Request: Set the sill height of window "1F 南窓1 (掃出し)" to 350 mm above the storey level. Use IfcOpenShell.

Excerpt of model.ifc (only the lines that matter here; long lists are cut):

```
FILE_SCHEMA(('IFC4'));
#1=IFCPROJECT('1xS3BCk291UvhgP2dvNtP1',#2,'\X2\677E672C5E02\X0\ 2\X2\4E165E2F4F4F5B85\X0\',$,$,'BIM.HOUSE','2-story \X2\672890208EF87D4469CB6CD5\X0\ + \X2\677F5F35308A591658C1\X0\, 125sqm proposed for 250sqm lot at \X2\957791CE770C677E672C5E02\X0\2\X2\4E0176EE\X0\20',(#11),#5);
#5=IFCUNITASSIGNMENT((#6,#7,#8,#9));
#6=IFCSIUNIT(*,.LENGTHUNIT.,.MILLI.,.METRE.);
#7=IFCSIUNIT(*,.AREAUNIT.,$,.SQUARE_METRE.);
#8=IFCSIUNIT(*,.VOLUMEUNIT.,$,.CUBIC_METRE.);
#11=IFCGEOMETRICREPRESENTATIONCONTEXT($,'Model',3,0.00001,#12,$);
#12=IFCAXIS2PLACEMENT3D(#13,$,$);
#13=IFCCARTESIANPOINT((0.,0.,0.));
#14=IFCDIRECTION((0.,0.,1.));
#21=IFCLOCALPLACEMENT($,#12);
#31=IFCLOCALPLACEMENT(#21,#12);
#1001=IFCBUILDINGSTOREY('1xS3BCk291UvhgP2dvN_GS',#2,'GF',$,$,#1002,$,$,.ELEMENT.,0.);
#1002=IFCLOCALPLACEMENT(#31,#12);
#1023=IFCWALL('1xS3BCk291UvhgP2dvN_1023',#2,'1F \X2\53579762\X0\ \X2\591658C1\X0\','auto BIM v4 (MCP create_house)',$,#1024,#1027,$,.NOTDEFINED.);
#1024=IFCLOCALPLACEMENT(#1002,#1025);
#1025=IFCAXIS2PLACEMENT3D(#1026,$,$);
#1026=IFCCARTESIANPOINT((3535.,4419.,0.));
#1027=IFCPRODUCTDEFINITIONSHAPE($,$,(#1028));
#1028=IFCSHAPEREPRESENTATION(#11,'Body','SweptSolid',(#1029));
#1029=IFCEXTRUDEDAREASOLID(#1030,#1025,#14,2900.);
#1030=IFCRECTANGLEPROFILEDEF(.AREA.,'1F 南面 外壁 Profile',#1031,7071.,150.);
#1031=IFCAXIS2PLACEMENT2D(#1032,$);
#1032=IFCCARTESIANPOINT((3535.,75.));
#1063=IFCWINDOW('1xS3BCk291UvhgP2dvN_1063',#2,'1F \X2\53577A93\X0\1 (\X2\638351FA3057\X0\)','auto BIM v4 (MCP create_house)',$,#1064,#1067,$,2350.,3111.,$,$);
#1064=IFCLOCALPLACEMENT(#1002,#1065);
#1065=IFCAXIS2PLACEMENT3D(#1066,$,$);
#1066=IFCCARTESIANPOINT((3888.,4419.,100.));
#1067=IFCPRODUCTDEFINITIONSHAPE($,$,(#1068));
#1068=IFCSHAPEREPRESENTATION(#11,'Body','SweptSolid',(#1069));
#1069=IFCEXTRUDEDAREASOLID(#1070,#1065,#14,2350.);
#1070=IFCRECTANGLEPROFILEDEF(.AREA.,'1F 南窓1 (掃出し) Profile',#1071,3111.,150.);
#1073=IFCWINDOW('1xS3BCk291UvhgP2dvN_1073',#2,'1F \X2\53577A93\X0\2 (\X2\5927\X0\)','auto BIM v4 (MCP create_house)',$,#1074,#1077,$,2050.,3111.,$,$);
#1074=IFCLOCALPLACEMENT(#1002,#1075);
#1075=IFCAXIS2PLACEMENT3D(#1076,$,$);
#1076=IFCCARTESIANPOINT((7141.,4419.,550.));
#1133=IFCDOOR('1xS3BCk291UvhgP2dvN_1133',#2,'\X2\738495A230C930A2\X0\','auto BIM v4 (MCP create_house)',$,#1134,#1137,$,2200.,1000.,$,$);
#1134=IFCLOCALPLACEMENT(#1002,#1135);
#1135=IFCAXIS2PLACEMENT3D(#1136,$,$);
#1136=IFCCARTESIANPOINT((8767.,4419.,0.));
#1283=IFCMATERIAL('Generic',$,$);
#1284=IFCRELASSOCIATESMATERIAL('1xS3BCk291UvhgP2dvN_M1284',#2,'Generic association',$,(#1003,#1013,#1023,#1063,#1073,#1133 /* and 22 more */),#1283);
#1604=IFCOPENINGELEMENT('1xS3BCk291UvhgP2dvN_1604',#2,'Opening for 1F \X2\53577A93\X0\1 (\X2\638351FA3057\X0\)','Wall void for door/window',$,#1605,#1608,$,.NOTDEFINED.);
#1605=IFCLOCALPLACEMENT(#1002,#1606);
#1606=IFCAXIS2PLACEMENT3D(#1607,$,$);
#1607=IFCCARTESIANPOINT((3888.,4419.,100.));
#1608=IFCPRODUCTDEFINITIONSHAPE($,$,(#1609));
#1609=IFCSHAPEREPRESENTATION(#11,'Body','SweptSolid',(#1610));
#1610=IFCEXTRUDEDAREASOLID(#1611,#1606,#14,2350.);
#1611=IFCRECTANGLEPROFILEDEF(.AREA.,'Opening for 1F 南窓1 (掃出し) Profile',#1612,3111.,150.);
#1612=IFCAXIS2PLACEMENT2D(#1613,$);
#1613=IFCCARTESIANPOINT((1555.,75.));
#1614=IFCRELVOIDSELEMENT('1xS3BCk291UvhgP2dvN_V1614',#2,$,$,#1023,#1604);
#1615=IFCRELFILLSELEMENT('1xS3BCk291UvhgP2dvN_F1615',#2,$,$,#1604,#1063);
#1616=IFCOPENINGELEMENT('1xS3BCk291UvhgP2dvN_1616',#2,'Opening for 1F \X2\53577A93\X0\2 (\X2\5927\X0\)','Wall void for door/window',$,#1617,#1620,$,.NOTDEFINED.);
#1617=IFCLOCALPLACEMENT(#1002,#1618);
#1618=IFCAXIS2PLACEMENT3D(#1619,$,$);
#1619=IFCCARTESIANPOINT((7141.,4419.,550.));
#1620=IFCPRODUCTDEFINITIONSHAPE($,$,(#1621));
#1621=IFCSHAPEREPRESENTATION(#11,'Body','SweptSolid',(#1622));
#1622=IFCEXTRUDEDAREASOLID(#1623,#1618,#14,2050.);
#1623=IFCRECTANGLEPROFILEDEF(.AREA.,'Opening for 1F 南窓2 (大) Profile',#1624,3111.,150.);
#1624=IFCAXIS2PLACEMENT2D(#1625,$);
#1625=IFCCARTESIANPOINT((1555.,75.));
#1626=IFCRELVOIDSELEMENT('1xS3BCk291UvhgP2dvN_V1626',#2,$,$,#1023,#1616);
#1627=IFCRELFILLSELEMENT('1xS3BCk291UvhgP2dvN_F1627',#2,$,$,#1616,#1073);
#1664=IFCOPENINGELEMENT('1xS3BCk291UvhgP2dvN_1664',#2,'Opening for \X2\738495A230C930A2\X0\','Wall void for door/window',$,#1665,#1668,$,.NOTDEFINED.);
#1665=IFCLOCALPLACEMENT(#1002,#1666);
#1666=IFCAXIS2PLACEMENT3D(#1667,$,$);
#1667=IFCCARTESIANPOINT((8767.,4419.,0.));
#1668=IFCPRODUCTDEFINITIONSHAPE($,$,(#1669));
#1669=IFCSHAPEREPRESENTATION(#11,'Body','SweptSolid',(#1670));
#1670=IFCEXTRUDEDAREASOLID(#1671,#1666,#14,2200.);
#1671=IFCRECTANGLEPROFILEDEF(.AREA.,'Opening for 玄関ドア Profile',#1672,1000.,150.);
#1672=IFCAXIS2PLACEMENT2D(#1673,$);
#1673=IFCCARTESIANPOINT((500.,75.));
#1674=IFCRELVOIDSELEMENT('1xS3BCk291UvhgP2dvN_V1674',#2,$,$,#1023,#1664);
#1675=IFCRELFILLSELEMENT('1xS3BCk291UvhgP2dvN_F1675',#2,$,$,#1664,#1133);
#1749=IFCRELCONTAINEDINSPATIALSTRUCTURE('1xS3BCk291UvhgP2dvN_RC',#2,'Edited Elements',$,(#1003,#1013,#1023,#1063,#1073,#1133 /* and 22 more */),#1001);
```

```python
import numpy as np
import ifcopenshell
import ifcopenshell.api.geometry
import ifcopenshell.geom
import ifcopenshell.util.element
import ifcopenshell.util.placement
import ifcopenshell.util.shape
import ifcopenshell.util.unit

model = ifcopenshell.open("model.ifc")
unit_scale = ifcopenshell.util.unit.calculate_unit_scale(model)

window = model.by_id(1063)
opening = window.FillsVoids[0].RelatingOpeningElement
storey = ifcopenshell.util.element.get_container(window, ifc_class="IfcBuildingStorey")
level = ifcopenshell.util.placement.get_local_placement(storey.ObjectPlacement)[2, 3]

# The opening's origin need not be at the sill, so measure its lowest point.
shape = ifcopenshell.geom.create_shape(ifcopenshell.geom.settings(), opening)
bottom = ifcopenshell.util.shape.get_shape_bottom_elevation(shape, shape.geometry) / unit_scale
dz = level + 350.0 - bottom

shift = np.array([0.0, 0.0, dz])
# The window is not placed relative to its opening, so move both.
for product in (opening, window):
    matrix = ifcopenshell.util.placement.get_local_placement(product.ObjectPlacement)
    matrix[:3, 3] += shift
    ifcopenshell.api.geometry.edit_object_placement(model, product=product, matrix=matrix, is_si=False)

print(f"moved by {dz * unit_scale:+.3f} m")

model.write("model_v2.ifc")
```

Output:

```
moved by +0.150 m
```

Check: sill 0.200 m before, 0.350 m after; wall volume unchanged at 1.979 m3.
